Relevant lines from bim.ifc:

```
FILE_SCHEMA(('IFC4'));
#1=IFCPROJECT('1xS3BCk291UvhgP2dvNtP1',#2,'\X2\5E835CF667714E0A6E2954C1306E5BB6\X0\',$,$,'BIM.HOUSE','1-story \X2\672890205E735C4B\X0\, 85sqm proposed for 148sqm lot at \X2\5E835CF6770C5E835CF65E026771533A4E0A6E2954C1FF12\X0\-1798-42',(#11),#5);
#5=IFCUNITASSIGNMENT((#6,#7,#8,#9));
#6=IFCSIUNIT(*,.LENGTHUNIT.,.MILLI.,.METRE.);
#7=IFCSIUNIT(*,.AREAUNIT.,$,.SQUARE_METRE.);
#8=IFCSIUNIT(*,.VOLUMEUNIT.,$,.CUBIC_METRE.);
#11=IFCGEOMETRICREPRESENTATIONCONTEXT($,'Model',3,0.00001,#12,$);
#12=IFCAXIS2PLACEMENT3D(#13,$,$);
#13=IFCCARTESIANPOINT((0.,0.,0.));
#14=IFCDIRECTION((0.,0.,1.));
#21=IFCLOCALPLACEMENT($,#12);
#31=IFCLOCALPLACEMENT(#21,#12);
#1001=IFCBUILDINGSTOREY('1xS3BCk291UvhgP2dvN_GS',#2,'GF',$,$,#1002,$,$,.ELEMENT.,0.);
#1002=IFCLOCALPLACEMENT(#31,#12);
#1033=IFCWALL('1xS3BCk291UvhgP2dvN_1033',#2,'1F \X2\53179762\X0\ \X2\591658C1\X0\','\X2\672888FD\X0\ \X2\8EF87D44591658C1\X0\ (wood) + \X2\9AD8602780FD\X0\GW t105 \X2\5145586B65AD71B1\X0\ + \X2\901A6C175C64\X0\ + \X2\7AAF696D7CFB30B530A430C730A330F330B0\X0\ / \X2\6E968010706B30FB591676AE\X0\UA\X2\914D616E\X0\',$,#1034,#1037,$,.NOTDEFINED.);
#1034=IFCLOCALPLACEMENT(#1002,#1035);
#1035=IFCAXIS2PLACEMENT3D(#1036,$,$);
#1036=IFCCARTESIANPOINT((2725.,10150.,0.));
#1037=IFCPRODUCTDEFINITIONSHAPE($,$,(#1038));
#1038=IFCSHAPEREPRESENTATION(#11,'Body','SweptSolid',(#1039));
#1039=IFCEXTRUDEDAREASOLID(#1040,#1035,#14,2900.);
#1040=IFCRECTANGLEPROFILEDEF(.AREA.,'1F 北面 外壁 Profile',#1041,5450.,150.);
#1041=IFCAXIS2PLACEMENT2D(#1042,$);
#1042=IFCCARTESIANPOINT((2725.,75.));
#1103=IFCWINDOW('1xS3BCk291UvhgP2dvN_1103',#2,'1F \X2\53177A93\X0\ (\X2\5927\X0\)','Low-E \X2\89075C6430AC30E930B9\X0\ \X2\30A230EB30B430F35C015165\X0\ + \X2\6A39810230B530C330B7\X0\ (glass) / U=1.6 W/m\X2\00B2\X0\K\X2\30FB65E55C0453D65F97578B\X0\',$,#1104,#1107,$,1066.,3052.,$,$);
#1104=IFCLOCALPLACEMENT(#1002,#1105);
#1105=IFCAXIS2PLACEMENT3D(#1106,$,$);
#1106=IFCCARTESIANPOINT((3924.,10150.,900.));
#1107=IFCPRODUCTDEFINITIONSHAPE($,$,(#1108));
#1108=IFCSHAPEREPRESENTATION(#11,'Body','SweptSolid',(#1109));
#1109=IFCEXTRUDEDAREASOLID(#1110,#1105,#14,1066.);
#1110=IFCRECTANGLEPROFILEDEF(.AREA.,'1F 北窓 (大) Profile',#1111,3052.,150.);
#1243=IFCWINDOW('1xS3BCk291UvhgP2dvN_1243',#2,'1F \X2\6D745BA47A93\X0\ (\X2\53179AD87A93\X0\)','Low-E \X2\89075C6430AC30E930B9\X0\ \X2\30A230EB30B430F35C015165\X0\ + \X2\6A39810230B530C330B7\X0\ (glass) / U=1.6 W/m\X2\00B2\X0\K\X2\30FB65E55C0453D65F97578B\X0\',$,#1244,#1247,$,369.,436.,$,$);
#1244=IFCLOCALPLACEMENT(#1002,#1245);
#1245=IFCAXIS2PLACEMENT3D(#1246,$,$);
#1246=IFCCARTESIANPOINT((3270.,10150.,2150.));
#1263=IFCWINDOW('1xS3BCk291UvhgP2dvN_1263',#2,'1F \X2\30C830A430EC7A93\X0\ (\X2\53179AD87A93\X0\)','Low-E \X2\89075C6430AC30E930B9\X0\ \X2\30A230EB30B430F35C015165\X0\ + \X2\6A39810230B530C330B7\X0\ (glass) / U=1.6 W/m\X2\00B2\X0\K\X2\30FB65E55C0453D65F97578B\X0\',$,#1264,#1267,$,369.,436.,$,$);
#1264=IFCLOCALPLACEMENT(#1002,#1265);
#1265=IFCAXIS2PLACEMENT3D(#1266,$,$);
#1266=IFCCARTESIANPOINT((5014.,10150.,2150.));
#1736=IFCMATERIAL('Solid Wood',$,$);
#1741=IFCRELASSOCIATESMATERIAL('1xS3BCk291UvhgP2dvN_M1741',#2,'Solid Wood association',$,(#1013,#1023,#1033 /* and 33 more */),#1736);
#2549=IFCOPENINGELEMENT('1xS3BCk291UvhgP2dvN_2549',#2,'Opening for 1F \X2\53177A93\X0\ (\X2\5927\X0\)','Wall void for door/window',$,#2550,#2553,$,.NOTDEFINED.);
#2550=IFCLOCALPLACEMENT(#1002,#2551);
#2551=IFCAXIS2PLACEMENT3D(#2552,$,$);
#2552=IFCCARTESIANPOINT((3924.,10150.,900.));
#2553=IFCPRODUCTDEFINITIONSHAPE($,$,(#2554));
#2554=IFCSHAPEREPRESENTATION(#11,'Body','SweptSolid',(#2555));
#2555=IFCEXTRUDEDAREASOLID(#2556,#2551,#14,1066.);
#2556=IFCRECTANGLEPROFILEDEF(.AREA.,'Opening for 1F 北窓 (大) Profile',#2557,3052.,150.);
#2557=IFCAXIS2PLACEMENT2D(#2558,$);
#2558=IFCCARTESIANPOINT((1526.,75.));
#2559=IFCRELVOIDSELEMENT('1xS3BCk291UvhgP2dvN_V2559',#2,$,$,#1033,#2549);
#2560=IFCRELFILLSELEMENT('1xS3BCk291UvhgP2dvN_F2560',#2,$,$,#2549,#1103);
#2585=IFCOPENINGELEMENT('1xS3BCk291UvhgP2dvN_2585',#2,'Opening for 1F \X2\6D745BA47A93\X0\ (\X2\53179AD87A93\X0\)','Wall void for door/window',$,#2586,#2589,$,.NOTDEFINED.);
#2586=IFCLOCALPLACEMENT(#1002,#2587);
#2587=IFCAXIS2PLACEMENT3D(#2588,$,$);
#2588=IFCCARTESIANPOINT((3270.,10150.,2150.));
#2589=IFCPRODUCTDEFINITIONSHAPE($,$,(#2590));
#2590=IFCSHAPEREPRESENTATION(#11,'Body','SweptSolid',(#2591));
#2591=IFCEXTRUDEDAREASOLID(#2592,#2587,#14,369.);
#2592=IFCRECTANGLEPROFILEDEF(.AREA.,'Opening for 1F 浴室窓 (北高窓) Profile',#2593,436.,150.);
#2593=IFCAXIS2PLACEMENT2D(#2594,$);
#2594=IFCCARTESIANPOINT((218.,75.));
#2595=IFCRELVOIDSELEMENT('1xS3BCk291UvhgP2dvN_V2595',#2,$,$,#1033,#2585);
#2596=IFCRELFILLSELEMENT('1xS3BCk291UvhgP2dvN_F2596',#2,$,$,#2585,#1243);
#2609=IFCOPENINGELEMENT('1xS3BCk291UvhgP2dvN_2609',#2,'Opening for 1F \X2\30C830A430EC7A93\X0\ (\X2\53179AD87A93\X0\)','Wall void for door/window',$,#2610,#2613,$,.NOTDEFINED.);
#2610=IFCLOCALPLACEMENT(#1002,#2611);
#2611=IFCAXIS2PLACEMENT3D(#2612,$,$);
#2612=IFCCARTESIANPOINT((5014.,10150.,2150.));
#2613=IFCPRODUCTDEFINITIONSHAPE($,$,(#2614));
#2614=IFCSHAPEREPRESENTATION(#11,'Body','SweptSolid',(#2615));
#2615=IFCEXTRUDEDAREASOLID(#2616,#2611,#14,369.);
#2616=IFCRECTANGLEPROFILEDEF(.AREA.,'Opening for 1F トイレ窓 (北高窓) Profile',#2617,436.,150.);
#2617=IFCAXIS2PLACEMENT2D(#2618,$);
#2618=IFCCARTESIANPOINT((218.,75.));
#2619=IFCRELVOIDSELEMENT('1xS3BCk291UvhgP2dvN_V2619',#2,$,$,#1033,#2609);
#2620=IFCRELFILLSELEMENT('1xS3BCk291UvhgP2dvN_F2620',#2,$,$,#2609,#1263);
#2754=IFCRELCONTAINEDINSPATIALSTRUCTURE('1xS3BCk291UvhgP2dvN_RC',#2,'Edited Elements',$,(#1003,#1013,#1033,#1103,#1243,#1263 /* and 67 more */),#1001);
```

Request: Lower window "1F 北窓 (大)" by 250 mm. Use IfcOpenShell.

```python
import numpy as np
import ifcopenshell
import ifcopenshell.api.geometry
import ifcopenshell.util.placement
import ifcopenshell.util.unit

model = ifcopenshell.open("bim.ifc")
unit_scale = ifcopenshell.util.unit.calculate_unit_scale(model)

window = model.by_guid("1xS3BCk291UvhgP2dvN_1103")
opening = window.FillsVoids[0].RelatingOpeningElement
dz = -250.0

shift = np.array([0.0, 0.0, dz])
# The window is not placed relative to its opening, so move both.
for product in (opening, window):
    matrix = ifcopenshell.util.placement.get_local_placement(product.ObjectPlacement)
    matrix[:3, 3] += shift
    ifcopenshell.api.geometry.edit_object_placement(model, product=product, matrix=matrix, is_si=False)

print(f"moved by {dz * unit_scale:+.3f} m")

model.write("bim_updated.ifc")
```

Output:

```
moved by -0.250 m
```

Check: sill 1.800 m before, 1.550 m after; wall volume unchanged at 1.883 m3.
